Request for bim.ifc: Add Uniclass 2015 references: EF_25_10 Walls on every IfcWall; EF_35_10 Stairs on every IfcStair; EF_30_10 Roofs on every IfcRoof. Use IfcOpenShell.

First a look at what the model holds.

```python
import ifcopenshell

model = ifcopenshell.open("bim.ifc")
print(model.schema)
print("classifications:", [c.Name for c in model.by_type("IfcClassification")])
for ifc_class in ("IfcDoor", "IfcRoof", "IfcStair", "IfcWall", "IfcWindow"):
    print(ifc_class, len(model.by_type(ifc_class)))
```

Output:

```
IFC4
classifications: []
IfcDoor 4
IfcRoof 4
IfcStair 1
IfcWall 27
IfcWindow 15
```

```python
import ifcopenshell
import ifcopenshell.api.classification

model = ifcopenshell.open("bim.ifc")

system = ifcopenshell.api.classification.add_classification(model, classification="Uniclass 2015")

codes = {
    "IfcWall": ("EF_25_10", "Walls"),
    "IfcStair": ("EF_35_10", "Stairs"),
    "IfcRoof": ("EF_30_10", "Roofs"),
}
for ifc_class, (code, name) in codes.items():
    products = model.by_type(ifc_class)
    ifcopenshell.api.classification.add_reference(
        model, products=products, classification=system, identification=code, name=name
    )
    print(code, len(products))

model.write("bim-out.ifc")
```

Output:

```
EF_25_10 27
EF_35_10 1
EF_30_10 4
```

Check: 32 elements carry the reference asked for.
